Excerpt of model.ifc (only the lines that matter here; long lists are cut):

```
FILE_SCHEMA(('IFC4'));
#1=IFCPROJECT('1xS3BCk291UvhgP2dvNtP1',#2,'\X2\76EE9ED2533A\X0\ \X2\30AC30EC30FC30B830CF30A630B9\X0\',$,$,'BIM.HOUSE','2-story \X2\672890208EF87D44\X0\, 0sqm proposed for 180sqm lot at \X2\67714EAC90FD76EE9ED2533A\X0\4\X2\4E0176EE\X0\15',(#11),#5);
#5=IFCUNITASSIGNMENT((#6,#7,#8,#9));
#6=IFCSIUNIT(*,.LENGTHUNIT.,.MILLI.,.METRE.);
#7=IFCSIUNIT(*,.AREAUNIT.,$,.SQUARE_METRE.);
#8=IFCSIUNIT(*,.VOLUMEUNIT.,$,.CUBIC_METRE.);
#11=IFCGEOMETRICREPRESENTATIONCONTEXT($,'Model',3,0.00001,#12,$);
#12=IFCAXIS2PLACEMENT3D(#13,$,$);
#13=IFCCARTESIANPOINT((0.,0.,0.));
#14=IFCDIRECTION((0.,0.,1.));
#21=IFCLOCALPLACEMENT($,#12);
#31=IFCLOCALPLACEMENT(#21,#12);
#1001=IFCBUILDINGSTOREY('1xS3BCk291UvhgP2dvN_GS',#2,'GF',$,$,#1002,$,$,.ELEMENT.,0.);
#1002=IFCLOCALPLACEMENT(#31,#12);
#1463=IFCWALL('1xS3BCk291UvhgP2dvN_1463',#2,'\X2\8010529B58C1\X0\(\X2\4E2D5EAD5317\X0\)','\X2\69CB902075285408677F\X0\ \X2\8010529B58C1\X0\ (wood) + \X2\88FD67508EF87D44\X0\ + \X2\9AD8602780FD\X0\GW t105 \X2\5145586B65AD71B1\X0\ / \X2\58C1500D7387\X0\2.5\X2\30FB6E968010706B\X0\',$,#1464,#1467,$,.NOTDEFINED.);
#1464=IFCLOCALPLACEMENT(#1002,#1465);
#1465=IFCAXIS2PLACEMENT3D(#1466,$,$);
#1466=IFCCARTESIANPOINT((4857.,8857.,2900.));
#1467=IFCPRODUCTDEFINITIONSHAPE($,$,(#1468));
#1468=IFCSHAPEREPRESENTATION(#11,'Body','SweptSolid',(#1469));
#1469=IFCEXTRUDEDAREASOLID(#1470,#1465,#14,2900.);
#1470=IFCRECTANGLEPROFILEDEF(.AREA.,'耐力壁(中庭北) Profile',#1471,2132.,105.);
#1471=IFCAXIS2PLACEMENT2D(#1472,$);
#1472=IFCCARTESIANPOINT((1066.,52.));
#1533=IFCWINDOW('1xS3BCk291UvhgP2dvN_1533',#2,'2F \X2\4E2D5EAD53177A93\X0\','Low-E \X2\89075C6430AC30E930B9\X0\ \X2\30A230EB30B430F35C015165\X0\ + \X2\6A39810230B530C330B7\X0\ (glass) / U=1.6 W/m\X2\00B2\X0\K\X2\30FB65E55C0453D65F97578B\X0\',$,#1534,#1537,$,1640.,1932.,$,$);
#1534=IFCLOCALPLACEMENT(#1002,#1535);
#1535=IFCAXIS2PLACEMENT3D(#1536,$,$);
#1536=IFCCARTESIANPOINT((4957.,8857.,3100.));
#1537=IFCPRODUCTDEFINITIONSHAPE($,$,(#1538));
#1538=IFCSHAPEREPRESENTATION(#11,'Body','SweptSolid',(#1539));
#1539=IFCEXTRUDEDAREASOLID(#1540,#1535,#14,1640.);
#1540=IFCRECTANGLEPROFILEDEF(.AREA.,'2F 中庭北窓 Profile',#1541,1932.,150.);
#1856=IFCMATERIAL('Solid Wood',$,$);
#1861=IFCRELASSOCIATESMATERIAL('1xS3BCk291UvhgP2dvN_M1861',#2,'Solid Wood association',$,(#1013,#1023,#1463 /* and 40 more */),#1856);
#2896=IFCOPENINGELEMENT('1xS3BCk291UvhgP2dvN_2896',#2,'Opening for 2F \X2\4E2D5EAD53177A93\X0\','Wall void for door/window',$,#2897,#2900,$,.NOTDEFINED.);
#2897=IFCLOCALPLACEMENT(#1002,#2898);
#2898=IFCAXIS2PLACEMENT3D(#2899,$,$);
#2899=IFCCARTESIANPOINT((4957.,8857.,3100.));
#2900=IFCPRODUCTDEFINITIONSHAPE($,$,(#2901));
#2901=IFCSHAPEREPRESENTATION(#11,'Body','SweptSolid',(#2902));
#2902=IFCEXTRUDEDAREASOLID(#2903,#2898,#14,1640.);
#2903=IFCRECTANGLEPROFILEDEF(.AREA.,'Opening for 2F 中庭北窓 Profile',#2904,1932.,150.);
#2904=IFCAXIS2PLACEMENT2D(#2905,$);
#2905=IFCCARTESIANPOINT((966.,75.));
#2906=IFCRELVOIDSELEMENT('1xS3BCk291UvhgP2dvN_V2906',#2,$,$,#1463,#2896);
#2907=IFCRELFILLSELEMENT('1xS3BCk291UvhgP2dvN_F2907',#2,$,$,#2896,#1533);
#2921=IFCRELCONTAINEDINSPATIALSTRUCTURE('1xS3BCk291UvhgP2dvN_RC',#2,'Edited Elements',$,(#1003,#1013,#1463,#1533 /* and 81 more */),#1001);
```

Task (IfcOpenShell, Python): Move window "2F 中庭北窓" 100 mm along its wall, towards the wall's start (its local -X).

```python
import ifcopenshell
import ifcopenshell.api.geometry
import ifcopenshell.util.placement
import ifcopenshell.util.unit

model = ifcopenshell.open("model.ifc")
unit_scale = ifcopenshell.util.unit.calculate_unit_scale(model)

window = model.by_guid("1xS3BCk291UvhgP2dvN_1533")
opening = window.FillsVoids[0].RelatingOpeningElement
wall = opening.VoidsElements[0].RelatingBuildingElement

wall_matrix = ifcopenshell.util.placement.get_local_placement(wall.ObjectPlacement)
shift = wall_matrix[:3, 0] * -0.1 / unit_scale
before = ifcopenshell.util.placement.get_local_placement(window.ObjectPlacement)[:3, 3].copy()

# The window is not placed relative to its opening, so move both.
for product in (opening, window):
    matrix = ifcopenshell.util.placement.get_local_placement(product.ObjectPlacement)
    matrix[:3, 3] += shift
    ifcopenshell.api.geometry.edit_object_placement(model, product=product, matrix=matrix, is_si=False)

after = ifcopenshell.util.placement.get_local_placement(window.ObjectPlacement)[:3, 3]
print("window moved by", (after - before).round(3) + 0.0)

model.write("model_rev.ifc")
```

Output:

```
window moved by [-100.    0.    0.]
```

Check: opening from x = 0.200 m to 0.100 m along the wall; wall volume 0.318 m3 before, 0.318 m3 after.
